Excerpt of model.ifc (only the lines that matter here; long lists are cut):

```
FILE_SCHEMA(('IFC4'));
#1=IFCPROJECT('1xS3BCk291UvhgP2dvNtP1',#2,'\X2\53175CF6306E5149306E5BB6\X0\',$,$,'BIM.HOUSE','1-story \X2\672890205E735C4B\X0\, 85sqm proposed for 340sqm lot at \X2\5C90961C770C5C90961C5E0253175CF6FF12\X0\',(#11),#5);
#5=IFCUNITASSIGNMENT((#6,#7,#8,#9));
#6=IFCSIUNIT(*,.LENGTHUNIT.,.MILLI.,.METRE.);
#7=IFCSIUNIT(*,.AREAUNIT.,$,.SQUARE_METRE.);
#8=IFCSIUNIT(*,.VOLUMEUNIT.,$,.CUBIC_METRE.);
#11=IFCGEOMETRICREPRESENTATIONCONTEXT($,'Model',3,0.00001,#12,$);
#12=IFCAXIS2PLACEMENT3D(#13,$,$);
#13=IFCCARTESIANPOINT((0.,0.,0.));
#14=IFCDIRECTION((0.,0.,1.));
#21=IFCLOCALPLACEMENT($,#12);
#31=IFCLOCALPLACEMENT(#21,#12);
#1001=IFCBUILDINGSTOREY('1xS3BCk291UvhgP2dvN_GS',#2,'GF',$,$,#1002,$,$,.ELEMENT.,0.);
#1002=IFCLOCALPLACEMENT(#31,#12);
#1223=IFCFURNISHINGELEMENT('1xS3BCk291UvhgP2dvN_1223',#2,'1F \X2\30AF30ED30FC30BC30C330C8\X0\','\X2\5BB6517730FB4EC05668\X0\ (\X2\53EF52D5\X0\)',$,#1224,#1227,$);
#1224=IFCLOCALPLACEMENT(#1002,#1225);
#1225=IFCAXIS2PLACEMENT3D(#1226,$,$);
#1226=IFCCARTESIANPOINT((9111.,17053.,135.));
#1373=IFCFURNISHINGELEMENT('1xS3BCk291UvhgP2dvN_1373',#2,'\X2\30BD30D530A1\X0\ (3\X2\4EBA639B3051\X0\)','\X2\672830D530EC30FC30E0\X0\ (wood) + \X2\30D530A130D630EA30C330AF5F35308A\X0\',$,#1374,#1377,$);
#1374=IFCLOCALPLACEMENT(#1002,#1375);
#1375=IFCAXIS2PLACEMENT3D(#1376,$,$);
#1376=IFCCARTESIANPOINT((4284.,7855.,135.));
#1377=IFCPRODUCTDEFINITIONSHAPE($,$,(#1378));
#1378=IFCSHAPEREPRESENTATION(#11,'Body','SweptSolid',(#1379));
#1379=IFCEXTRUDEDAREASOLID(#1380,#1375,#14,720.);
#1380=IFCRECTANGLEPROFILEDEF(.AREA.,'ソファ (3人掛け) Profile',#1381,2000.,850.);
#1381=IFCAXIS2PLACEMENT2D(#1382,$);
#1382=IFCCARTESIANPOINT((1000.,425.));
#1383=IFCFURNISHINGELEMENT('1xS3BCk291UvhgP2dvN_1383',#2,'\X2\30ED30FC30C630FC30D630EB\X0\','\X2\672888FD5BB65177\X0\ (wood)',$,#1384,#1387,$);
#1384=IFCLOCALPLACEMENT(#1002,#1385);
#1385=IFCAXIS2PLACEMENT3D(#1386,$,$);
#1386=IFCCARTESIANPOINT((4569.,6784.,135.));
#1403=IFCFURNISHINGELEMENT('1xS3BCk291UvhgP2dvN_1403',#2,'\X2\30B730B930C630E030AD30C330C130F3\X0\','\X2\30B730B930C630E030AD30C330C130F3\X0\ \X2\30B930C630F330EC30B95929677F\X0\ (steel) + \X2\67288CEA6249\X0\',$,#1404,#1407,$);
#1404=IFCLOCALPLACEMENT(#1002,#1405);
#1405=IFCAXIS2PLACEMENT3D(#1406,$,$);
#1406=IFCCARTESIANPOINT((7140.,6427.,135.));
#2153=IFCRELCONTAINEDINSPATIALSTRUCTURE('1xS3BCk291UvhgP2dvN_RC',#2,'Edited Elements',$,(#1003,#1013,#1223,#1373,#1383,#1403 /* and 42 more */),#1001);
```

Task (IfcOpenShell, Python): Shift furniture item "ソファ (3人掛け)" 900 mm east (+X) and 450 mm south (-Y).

```python
import ifcopenshell
import ifcopenshell.api.geometry
import ifcopenshell.util.placement

model = ifcopenshell.open("model.ifc")

item = model.by_guid("1xS3BCk291UvhgP2dvN_1373")
matrix = ifcopenshell.util.placement.get_local_placement(item.ObjectPlacement)
matrix[0, 3] += 900.0
matrix[1, 3] -= 450.0
ifcopenshell.api.geometry.edit_object_placement(model, product=item, matrix=matrix, is_si=False)

print(ifcopenshell.util.placement.get_local_placement(item.ObjectPlacement).round(3) + 0.0)

model.write("model_rev.ifc")
```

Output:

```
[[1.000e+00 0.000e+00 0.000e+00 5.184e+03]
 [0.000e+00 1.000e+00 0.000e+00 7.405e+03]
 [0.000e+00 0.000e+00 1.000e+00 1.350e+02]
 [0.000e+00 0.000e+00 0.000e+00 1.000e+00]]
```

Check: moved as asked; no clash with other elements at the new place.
